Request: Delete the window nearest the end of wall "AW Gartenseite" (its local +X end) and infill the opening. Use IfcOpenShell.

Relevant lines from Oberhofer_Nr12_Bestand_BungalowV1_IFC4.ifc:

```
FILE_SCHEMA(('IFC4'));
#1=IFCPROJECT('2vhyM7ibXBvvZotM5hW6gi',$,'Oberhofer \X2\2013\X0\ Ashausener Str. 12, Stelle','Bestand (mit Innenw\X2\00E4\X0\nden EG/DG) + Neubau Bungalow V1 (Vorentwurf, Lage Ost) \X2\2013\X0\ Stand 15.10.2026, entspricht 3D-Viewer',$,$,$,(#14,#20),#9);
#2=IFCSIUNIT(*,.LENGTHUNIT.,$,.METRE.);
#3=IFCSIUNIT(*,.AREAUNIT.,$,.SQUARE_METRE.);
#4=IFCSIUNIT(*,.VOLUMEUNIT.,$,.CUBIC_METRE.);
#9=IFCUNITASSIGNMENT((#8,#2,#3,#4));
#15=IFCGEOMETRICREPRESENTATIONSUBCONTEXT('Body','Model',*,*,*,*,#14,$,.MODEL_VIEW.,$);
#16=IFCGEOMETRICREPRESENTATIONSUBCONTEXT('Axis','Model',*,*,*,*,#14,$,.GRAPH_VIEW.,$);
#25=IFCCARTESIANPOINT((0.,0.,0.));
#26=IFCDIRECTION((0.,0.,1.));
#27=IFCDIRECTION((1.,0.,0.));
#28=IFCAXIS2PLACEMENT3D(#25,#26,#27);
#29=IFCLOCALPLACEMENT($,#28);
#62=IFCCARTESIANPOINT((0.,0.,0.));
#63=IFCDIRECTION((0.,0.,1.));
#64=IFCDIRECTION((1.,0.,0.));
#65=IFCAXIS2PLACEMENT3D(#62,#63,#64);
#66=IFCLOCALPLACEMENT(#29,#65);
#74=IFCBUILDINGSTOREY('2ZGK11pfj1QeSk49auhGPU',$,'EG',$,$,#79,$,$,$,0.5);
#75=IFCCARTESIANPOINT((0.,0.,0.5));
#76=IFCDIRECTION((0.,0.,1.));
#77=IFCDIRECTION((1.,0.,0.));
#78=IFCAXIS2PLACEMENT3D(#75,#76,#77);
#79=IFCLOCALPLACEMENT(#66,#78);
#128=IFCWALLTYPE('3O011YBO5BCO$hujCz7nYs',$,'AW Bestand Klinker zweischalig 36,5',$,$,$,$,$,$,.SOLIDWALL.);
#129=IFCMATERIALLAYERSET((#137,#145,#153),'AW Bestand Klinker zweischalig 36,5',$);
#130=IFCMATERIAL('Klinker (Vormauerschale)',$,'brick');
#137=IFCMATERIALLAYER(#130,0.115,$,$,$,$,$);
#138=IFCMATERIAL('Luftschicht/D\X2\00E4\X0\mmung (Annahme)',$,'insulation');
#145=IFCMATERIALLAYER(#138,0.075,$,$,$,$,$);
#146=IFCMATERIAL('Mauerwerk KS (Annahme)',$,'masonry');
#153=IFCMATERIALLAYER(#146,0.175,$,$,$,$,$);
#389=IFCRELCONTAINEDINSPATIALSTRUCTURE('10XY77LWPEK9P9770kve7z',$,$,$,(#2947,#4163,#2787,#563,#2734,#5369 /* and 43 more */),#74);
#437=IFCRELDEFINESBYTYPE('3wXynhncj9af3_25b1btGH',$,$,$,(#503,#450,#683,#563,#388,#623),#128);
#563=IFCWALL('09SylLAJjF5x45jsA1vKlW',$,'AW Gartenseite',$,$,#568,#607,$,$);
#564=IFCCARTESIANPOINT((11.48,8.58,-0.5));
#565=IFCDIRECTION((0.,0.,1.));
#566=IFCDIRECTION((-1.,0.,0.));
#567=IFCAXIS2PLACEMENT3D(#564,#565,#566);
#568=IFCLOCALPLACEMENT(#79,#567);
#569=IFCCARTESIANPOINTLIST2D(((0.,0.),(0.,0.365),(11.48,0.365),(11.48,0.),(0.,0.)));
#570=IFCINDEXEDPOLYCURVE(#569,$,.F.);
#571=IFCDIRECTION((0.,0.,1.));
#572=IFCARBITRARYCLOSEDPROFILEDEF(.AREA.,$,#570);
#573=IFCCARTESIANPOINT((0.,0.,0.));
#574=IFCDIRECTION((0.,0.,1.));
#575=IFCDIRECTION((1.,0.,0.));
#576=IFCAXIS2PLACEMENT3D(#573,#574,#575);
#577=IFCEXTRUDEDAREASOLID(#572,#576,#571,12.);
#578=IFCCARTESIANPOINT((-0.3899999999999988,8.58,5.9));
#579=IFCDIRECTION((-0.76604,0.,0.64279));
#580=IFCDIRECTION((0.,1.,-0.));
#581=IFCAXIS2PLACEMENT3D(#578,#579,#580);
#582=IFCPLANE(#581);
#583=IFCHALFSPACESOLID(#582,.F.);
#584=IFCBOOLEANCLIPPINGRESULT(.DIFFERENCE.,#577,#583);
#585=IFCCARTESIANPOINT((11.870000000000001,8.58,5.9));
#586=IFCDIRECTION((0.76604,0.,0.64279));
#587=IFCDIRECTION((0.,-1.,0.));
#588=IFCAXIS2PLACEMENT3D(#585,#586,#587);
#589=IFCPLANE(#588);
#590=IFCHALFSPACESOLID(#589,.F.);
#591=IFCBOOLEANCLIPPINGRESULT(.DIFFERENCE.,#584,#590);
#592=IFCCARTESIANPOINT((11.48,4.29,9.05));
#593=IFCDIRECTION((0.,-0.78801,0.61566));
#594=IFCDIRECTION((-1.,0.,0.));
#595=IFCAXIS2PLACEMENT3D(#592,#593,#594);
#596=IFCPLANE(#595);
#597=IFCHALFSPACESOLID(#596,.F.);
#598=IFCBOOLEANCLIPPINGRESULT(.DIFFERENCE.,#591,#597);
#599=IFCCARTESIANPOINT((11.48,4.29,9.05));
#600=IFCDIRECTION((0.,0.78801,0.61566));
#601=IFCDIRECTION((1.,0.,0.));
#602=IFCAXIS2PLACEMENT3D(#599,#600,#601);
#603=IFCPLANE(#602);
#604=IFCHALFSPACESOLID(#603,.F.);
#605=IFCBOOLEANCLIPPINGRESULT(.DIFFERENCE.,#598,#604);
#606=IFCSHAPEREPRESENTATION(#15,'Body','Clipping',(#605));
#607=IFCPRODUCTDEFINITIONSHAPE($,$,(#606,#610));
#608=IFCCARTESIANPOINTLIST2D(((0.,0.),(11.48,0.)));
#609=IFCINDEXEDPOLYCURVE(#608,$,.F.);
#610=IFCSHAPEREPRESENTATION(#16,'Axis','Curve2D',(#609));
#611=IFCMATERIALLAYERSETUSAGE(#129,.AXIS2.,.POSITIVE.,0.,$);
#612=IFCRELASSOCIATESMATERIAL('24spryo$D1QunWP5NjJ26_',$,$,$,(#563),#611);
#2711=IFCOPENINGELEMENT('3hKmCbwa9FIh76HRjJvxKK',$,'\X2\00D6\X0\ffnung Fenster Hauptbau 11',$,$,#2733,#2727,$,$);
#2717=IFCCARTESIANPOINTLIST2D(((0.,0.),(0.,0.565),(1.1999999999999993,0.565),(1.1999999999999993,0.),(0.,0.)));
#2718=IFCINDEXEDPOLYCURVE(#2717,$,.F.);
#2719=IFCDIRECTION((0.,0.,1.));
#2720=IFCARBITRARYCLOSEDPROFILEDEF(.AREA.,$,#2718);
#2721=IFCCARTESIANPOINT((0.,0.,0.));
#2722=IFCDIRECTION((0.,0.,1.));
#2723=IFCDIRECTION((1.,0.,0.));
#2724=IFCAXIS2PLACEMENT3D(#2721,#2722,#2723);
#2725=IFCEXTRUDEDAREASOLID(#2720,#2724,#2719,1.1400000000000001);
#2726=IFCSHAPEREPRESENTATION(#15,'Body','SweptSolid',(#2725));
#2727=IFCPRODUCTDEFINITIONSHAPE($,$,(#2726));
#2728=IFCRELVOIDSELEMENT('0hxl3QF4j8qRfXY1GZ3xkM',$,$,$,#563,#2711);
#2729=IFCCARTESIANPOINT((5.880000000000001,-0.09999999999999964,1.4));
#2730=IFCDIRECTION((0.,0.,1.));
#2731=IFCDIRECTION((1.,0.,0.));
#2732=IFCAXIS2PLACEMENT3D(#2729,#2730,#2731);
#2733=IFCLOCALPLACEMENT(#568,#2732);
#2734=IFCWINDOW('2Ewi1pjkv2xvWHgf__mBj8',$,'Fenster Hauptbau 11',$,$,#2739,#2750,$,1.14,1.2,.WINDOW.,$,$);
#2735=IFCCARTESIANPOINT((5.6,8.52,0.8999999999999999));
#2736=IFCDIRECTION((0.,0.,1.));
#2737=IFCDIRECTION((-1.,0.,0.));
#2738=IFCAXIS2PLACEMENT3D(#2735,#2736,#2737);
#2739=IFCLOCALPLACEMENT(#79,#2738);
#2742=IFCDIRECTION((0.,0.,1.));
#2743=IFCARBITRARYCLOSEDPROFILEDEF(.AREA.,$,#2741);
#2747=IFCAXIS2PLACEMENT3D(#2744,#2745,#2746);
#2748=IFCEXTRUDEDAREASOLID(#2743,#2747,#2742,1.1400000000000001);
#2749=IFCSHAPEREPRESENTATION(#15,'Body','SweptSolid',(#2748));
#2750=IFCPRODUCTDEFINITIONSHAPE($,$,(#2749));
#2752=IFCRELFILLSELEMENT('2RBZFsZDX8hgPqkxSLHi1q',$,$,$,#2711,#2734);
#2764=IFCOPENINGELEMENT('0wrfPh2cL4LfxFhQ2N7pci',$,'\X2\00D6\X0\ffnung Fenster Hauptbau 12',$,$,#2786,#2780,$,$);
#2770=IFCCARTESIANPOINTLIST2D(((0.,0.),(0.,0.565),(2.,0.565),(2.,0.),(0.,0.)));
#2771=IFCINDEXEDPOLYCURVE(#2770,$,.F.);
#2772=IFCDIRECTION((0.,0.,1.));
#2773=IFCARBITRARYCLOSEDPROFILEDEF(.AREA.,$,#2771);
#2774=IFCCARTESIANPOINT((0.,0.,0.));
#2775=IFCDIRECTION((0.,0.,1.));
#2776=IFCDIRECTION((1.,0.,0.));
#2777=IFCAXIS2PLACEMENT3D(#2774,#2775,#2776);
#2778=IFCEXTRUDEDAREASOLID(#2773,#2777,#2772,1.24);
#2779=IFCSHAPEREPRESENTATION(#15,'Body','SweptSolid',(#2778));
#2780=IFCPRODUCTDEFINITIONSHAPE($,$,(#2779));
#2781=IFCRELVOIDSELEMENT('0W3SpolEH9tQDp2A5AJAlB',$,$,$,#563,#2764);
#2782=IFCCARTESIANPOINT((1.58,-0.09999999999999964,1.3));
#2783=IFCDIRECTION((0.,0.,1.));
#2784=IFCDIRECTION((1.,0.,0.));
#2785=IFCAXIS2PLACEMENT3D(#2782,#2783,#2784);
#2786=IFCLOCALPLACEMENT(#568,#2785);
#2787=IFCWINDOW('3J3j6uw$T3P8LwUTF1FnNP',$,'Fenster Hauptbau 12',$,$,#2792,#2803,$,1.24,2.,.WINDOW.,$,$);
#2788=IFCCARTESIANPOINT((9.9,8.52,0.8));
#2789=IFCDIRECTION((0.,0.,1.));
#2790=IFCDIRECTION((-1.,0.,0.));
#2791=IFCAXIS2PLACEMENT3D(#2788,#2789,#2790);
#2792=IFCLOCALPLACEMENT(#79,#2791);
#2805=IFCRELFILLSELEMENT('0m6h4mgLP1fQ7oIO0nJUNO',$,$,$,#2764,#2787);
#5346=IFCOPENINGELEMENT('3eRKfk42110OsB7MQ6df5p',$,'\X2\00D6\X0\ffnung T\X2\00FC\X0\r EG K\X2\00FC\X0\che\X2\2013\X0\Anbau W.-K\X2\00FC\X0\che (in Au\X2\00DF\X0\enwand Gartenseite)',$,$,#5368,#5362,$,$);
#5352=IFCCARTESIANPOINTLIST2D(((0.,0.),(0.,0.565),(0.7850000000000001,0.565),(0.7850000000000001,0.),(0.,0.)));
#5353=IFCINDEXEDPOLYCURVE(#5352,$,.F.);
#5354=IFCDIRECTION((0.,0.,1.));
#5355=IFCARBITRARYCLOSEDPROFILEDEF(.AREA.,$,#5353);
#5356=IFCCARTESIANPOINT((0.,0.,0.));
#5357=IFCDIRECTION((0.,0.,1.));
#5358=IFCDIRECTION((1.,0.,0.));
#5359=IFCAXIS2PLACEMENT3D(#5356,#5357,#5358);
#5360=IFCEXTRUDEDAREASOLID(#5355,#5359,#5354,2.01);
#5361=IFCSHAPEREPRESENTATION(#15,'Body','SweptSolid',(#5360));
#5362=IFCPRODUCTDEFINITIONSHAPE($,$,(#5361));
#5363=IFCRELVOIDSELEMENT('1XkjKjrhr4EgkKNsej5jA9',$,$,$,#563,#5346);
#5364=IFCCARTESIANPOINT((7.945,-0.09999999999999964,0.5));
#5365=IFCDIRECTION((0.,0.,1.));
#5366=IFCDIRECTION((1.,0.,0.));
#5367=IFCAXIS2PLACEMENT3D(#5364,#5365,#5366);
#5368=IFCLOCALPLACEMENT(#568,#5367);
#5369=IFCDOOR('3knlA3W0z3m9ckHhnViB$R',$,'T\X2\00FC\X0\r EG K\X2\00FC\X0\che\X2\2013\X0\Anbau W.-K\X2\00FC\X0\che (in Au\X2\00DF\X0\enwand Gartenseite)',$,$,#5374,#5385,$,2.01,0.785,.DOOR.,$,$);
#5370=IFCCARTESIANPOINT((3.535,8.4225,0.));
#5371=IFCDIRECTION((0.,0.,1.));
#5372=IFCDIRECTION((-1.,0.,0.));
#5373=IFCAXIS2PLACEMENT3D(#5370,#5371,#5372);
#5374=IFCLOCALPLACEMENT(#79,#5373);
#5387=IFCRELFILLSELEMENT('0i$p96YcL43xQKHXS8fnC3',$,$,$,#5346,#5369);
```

```python
import ifcopenshell
import ifcopenshell.api.feature
import ifcopenshell.api.root
import ifcopenshell.geom
import ifcopenshell.util.shape

model = ifcopenshell.open("Oberhofer_Nr12_Bestand_BungalowV1_IFC4.ifc")
settings = ifcopenshell.geom.settings()


def volume(element):
    """Net volume in cubic metres, openings subtracted."""
    shape = ifcopenshell.geom.create_shape(settings, element)
    return ifcopenshell.util.shape.get_volume(shape.geometry)


window = model.by_guid("2Ewi1pjkv2xvWHgf__mBj8")
opening = window.FillsVoids[0].RelatingOpeningElement
wall = opening.VoidsElements[0].RelatingBuildingElement
before = volume(wall)

ifcopenshell.api.root.remove_product(model, product=window)
ifcopenshell.api.feature.remove_feature(model, feature=opening)

after = volume(wall)

print(f"wall volume {before:.3f} -> {after:.3f} m3")

model.write("Oberhofer_Nr12_Bestand_BungalowV1_IFC4_edited.ifc")
```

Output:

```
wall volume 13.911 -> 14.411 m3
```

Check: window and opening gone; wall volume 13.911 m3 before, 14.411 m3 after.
